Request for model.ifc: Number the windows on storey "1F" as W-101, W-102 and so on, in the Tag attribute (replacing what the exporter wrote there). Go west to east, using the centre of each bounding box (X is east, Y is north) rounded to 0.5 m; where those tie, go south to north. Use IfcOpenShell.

First a look at what the model holds.

```python
import ifcopenshell
import ifcopenshell.util.element
import ifcopenshell.util.placement

model = ifcopenshell.open("model.ifc")
print(model.schema)
storey = next(s for s in model.by_type("IfcBuildingStorey") if s.Name == "1F")
windows = [e for e in ifcopenshell.util.element.get_decomposition(storey) if e.is_a("IfcWindow")]
for e in sorted(windows, key=lambda e: e.id()):
    origin = ifcopenshell.util.placement.get_local_placement(e.ObjectPlacement)[:3, 3]
    print(e.id(), e.Tag, e.Name, origin.round(2) + 0.0, sep=" | ")
```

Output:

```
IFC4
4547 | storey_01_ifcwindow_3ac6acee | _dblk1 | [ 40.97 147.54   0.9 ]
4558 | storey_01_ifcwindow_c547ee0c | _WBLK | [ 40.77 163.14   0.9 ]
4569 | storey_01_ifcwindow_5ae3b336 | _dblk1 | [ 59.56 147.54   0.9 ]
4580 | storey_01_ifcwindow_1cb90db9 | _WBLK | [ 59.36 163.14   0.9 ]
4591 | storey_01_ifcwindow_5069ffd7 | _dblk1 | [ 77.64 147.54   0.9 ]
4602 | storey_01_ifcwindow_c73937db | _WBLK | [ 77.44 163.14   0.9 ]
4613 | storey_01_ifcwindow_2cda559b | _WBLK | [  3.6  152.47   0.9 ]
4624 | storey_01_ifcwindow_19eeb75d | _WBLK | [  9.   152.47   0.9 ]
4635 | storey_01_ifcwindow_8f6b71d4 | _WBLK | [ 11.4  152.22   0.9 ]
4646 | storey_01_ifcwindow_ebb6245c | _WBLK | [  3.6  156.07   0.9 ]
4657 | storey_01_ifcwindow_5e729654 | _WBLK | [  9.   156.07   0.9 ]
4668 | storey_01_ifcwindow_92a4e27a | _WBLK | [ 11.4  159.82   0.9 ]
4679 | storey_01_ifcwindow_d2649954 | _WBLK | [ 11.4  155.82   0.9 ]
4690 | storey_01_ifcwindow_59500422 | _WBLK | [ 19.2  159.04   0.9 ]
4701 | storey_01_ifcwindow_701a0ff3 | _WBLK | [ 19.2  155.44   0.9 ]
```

```python
import ifcopenshell
import ifcopenshell.geom
import ifcopenshell.util.element
import ifcopenshell.util.shape

model = ifcopenshell.open("model.ifc")
settings = ifcopenshell.geom.settings()
settings.set("use-world-coords", True)


def centre(element):
    shape = ifcopenshell.geom.create_shape(settings, element)
    return ifcopenshell.util.shape.get_bbox_centroid(shape.geometry)


storey = next(s for s in model.by_type("IfcBuildingStorey") if s.Name == "1F")
windows = [e for e in ifcopenshell.util.element.get_decomposition(storey) if e.is_a("IfcWindow")]

# Insertion points can sit at a corner or the storey origin, so sort by the geometry (in metres).
centres = {e: centre(e) for e in windows}
windows.sort(key=lambda e: (round(centres[e][0] / 0.5), centres[e][1]))

for i, e in enumerate(windows, start=1):
    number = f"W-1{i:02d}"
    e.Tag = number
    print(e.id(), number)

model.write("model-out.ifc")
```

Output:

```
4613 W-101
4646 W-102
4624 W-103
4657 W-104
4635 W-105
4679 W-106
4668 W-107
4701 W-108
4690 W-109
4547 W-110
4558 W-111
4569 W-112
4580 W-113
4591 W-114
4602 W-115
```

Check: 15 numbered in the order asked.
